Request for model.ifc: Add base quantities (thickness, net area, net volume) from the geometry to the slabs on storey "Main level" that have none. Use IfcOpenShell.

First a look at what the model holds.

```python
import ifcopenshell
import ifcopenshell.util.element
import ifcopenshell.util.unit

model = ifcopenshell.open("model.ifc")
print(model.schema)
for unit_type in ("LENGTHUNIT", "AREAUNIT", "VOLUMEUNIT"):
    print(unit_type, ifcopenshell.util.unit.calculate_unit_scale(model, unit_type))
storey = next(s for s in model.by_type("IfcBuildingStorey") if s.Name == "Main level")
slabs = [e for e in ifcopenshell.util.element.get_decomposition(storey) if e.is_a("IfcSlab")]
for e in sorted(slabs, key=lambda e: e.id()):
    print(e.id(), e.is_a(), e.Name, list(ifcopenshell.util.element.get_psets(e, qtos_only=True)), sep=" | ")
```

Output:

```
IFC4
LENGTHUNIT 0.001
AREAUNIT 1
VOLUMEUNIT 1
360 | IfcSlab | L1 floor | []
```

```python
import ifcopenshell
import ifcopenshell.api.pset
import ifcopenshell.geom
import ifcopenshell.util.element
import ifcopenshell.util.shape
import ifcopenshell.util.unit

model = ifcopenshell.open("model.ifc")
unit_scale = ifcopenshell.util.unit.calculate_unit_scale(model)
area_scale = ifcopenshell.util.unit.calculate_unit_scale(model, "AREAUNIT")
volume_scale = ifcopenshell.util.unit.calculate_unit_scale(model, "VOLUMEUNIT")
settings = ifcopenshell.geom.settings()

storey = next(s for s in model.by_type("IfcBuildingStorey") if s.Name == "Main level")
slabs = [e for e in ifcopenshell.util.element.get_decomposition(storey) if e.is_a("IfcSlab")]

for e in sorted(slabs, key=lambda e: e.id()):
    if ifcopenshell.util.element.get_psets(e, qtos_only=True, should_inherit=False):
        continue
    # Geometry comes back in metres, in the element's own axes.
    shape = ifcopenshell.geom.create_shape(settings, e)
    values = {
        "Width": ifcopenshell.util.shape.get_z(shape.geometry) / unit_scale,
        "NetArea": ifcopenshell.util.shape.get_footprint_area(shape.geometry) / area_scale,
        "NetVolume": ifcopenshell.util.shape.get_volume(shape.geometry) / volume_scale,
    }
    qto = ifcopenshell.api.pset.add_qto(model, product=e, name="Qto_SlabBaseQuantities")
    ifcopenshell.api.pset.edit_qto(model, qto=qto, properties=values)
    print(e.id(), {k: round(v, 3) for k, v in values.items()})

model.write("model_rev.ifc")
```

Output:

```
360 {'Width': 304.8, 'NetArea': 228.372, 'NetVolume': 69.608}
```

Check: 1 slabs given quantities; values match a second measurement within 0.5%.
